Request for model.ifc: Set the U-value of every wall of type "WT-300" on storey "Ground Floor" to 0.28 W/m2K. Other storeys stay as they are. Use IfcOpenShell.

First a look at what the model holds.

```python
import ifcopenshell
import ifcopenshell.util.element

model = ifcopenshell.open("model.ifc")
print(model.schema)
storey = next(s for s in model.by_type("IfcBuildingStorey") if s.Name == "Ground Floor")
walls = [e for e in ifcopenshell.util.element.get_decomposition(storey) if e.is_a("IfcWall")]
seen = {}
for e in walls:
    element_type = ifcopenshell.util.element.get_type(e)
    key = (element_type.Name if element_type != e and element_type else None, ifcopenshell.util.element.get_pset(e, "Pset_WallCommon", "ThermalTransmittance"))
    seen[key] = seen.get(key, 0) + 1
for (name, value), count in sorted(seen.items(), key=str):
    print(count, "x", name, "|", value)
```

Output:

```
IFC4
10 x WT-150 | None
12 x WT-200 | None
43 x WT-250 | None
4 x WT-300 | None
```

```python
import ifcopenshell
import ifcopenshell.api.pset
import ifcopenshell.util.element

model = ifcopenshell.open("model.ifc")

storey = next(s for s in model.by_type("IfcBuildingStorey") if s.Name == "Ground Floor")
walls = [e for e in ifcopenshell.util.element.get_decomposition(storey) if e.is_a("IfcWall")]

count = 0
for e in walls:
    element_type = ifcopenshell.util.element.get_type(e)
    if element_type in (None, e) or element_type.Name != "WT-300":
        continue
    # add_pset returns the element's existing set when there is one.
    pset = ifcopenshell.api.pset.add_pset(model, product=e, name="Pset_WallCommon")
    ifcopenshell.api.pset.edit_pset(model, pset=pset, properties={"ThermalTransmittance": 0.28})
    count += 1

print(count, "walls updated")

model.write("model_v2.ifc")
```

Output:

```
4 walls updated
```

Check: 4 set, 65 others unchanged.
